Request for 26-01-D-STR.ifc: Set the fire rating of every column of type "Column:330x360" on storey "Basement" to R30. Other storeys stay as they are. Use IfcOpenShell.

First a look at what the model holds.

```python
import ifcopenshell
import ifcopenshell.util.element

model = ifcopenshell.open("26-01-D-STR.ifc")
print(model.schema)
storey = next(s for s in model.by_type("IfcBuildingStorey") if s.Name == "Basement")
columns = [e for e in ifcopenshell.util.element.get_decomposition(storey) if e.is_a("IfcColumn")]
seen = {}
for e in columns:
    element_type = ifcopenshell.util.element.get_type(e)
    key = (element_type.Name if element_type != e and element_type else None, ifcopenshell.util.element.get_pset(e, "Pset_ColumnCommon", "FireRating"))
    seen[key] = seen.get(key, 0) + 1
for (name, value), count in sorted(seen.items(), key=str):
    print(count, "x", name, "|", value)
```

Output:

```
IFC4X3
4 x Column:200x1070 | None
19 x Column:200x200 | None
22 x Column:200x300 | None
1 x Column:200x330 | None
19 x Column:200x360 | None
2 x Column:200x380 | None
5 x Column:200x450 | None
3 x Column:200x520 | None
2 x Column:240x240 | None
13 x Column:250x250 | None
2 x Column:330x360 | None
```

```python
import ifcopenshell
import ifcopenshell.api.pset
import ifcopenshell.util.element

model = ifcopenshell.open("26-01-D-STR.ifc")

storey = next(s for s in model.by_type("IfcBuildingStorey") if s.Name == "Basement")
columns = [e for e in ifcopenshell.util.element.get_decomposition(storey) if e.is_a("IfcColumn")]

count = 0
for e in columns:
    element_type = ifcopenshell.util.element.get_type(e)
    if element_type in (None, e) or element_type.Name != "Column:330x360":
        continue
    # add_pset returns the element's existing set when there is one.
    pset = ifcopenshell.api.pset.add_pset(model, product=e, name="Pset_ColumnCommon")
    ifcopenshell.api.pset.edit_pset(model, pset=pset, properties={"FireRating": "R30"})
    count += 1

print(count, "columns updated")

model.write("26-01-D-STR_updated.ifc")
```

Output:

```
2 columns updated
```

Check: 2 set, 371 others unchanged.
